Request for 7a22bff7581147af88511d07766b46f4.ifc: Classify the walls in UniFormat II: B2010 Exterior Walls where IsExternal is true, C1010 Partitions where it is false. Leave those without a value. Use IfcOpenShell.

First a look at what the model holds.

```python
import ifcopenshell
import ifcopenshell.util.element

model = ifcopenshell.open("7a22bff7581147af88511d07766b46f4.ifc")
print(model.schema)
print("classifications:", [c.Name for c in model.by_type("IfcClassification")])
values = [ifcopenshell.util.element.get_pset(e, "Pset_WallCommon", "IsExternal") for e in model.by_type("IfcWall")]
for value in (True, False, None):
    print("IsExternal", value, values.count(value))
```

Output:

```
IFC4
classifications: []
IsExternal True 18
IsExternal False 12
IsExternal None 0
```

```python
import ifcopenshell
import ifcopenshell.api.classification
import ifcopenshell.util.element

model = ifcopenshell.open("7a22bff7581147af88511d07766b46f4.ifc")

system = ifcopenshell.api.classification.add_classification(model, classification="UniFormat II")

walls = model.by_type("IfcWall")
external = {e: ifcopenshell.util.element.get_pset(e, "Pset_WallCommon", "IsExternal") for e in walls}
for flag, code, name in ((True, "B2010", "Exterior Walls"), (False, "C1010", "Partitions")):
    products = [e for e in walls if external[e] is flag]
    ifcopenshell.api.classification.add_reference(
        model, products=products, classification=system, identification=code, name=name
    )
    print(code, len(products))

model.write("7a22bff7581147af88511d07766b46f4-out.ifc")
```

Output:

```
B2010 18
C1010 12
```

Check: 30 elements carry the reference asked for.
